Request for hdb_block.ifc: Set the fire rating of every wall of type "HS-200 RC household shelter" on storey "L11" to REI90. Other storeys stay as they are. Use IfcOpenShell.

First a look at what the model holds.

```python
import ifcopenshell
import ifcopenshell.util.element

model = ifcopenshell.open("hdb_block.ifc")
print(model.schema)
storey = next(s for s in model.by_type("IfcBuildingStorey") if s.Name == "L11")
walls = [e for e in ifcopenshell.util.element.get_decomposition(storey) if e.is_a("IfcWall")]
seen = {}
for e in walls:
    element_type = ifcopenshell.util.element.get_type(e)
    key = (element_type.Name if element_type != e and element_type else None, ifcopenshell.util.element.get_pset(e, "Pset_WallCommon", "FireRating"))
    seen[key] = seen.get(key, 0) + 1
for (name, value), count in sorted(seen.items(), key=str):
    print(count, "x", name, "|", value)
```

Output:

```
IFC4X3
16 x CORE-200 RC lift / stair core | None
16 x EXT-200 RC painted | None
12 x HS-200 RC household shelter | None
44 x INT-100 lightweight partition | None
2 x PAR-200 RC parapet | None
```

```python
import ifcopenshell
import ifcopenshell.api.pset
import ifcopenshell.util.element

model = ifcopenshell.open("hdb_block.ifc")

storey = next(s for s in model.by_type("IfcBuildingStorey") if s.Name == "L11")
walls = [e for e in ifcopenshell.util.element.get_decomposition(storey) if e.is_a("IfcWall")]

count = 0
for e in walls:
    element_type = ifcopenshell.util.element.get_type(e)
    if element_type in (None, e) or element_type.Name != "HS-200 RC household shelter":
        continue
    # add_pset returns the element's existing set when there is one.
    pset = ifcopenshell.api.pset.add_pset(model, product=e, name="Pset_WallCommon")
    ifcopenshell.api.pset.edit_pset(model, pset=pset, properties={"FireRating": "REI90"})
    count += 1

print(count, "walls updated")

model.write("hdb_block-out.ifc")
```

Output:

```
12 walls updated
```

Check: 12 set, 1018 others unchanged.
